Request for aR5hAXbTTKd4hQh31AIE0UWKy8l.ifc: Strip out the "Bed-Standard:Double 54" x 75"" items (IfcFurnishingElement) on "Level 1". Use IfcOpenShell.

First a look at what the model holds.

```python
import ifcopenshell
import ifcopenshell.util.element

model = ifcopenshell.open("aR5hAXbTTKd4hQh31AIE0UWKy8l.ifc")
print(model.schema)
storey = next(s for s in model.by_type("IfcBuildingStorey") if s.Name == "Level 1")
furniture = [e for e in ifcopenshell.util.element.get_decomposition(storey) if e.is_a("IfcFurnishingElement")]
seen = {}
for e in furniture:
    element_type = ifcopenshell.util.element.get_type(e)
    name = element_type.Name if element_type not in (None, e) else None
    seen[name] = seen.get(name, 0) + 1
for name, count in sorted(seen.items(), key=str):
    print(count, "x", name)
```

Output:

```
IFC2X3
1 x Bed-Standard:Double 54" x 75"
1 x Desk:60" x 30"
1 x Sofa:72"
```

```python
import ifcopenshell
import ifcopenshell.api.root
import ifcopenshell.util.element

model = ifcopenshell.open("aR5hAXbTTKd4hQh31AIE0UWKy8l.ifc")

storey = next(s for s in model.by_type("IfcBuildingStorey") if s.Name == "Level 1")
furniture = [e for e in ifcopenshell.util.element.get_decomposition(storey) if e.is_a("IfcFurnishingElement")]
targets = [e for e in furniture if (t := ifcopenshell.util.element.get_type(e)) not in (None, e) and t.Name == 'Bed-Standard:Double 54" x 75"']

for e in targets:
    ifcopenshell.api.root.remove_product(model, product=e)
print(len(targets), "removed")

model.write("aR5hAXbTTKd4hQh31AIE0UWKy8l_v2.ifc")
```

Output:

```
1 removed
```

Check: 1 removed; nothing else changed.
